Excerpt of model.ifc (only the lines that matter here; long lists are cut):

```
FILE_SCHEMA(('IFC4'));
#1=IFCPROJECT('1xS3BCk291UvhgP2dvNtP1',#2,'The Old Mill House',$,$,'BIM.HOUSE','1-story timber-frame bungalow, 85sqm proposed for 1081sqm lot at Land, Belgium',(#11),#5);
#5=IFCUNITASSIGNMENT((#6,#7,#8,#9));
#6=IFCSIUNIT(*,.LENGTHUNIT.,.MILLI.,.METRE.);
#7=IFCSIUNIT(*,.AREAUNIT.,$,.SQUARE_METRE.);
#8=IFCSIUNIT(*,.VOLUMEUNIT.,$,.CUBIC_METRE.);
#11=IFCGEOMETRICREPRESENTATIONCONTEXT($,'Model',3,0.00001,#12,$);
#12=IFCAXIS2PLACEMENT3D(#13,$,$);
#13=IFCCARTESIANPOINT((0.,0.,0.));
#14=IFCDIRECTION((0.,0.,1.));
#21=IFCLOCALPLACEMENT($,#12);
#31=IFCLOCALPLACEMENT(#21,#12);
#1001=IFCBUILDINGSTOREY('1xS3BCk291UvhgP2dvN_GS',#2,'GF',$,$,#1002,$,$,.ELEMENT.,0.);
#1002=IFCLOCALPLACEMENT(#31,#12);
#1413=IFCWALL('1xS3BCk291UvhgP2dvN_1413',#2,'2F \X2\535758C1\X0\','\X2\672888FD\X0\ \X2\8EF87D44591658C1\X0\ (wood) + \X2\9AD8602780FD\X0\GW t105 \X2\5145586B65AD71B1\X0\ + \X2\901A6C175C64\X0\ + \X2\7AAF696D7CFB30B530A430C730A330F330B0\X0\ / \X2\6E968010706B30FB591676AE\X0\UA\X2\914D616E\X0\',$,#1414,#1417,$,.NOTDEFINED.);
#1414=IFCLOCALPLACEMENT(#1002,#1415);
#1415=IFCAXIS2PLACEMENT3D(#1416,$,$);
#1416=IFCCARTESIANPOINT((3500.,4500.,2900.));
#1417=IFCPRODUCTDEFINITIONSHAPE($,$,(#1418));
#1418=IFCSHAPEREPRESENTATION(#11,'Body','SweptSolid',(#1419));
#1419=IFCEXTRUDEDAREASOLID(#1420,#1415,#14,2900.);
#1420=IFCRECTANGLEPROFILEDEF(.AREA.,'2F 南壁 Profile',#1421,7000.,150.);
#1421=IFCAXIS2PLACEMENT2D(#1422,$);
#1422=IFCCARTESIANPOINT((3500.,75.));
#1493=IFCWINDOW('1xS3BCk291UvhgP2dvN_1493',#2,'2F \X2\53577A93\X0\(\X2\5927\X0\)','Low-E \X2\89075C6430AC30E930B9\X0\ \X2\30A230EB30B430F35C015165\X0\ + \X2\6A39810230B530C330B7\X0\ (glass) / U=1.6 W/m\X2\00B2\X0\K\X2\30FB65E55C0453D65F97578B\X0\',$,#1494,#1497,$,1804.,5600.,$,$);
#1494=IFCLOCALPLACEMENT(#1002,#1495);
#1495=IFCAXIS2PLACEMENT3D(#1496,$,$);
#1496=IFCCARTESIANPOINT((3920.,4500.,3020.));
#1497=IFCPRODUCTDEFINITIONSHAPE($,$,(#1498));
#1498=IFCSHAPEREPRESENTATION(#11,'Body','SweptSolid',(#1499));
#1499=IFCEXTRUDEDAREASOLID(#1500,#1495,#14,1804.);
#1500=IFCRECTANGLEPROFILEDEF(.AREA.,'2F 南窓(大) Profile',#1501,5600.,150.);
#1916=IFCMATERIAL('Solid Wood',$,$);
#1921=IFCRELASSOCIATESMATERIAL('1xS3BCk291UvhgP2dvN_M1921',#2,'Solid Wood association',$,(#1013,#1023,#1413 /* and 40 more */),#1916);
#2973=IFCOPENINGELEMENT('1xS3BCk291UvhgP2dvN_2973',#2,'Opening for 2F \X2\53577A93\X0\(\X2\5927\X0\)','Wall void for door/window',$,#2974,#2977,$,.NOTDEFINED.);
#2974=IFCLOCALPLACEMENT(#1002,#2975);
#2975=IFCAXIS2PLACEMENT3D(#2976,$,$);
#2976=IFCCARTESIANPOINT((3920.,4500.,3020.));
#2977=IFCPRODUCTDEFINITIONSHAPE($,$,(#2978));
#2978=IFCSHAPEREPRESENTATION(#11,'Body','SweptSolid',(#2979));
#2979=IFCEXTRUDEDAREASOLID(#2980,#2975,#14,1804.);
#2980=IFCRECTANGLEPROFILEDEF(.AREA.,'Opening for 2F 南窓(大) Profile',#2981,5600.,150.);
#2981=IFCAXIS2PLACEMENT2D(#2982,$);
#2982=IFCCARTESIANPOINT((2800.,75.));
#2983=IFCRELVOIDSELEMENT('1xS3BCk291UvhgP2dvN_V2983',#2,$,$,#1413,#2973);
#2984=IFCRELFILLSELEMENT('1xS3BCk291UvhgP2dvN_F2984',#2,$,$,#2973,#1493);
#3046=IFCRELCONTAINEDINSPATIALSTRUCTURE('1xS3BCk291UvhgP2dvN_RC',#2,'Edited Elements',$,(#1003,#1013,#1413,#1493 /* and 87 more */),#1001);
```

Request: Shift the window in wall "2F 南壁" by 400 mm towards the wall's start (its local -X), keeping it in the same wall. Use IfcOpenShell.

```python
import ifcopenshell
import ifcopenshell.api.geometry
import ifcopenshell.util.placement
import ifcopenshell.util.unit

model = ifcopenshell.open("model.ifc")
unit_scale = ifcopenshell.util.unit.calculate_unit_scale(model)

window = model.by_guid("1xS3BCk291UvhgP2dvN_1493")
opening = window.FillsVoids[0].RelatingOpeningElement
wall = opening.VoidsElements[0].RelatingBuildingElement

wall_matrix = ifcopenshell.util.placement.get_local_placement(wall.ObjectPlacement)
shift = wall_matrix[:3, 0] * -0.4 / unit_scale
before = ifcopenshell.util.placement.get_local_placement(window.ObjectPlacement)[:3, 3].copy()

# The window is not placed relative to its opening, so move both.
for product in (opening, window):
    matrix = ifcopenshell.util.placement.get_local_placement(product.ObjectPlacement)
    matrix[:3, 3] += shift
    ifcopenshell.api.geometry.edit_object_placement(model, product=product, matrix=matrix, is_si=False)

after = ifcopenshell.util.placement.get_local_placement(window.ObjectPlacement)[:3, 3]
print("window moved by", (after - before).round(3) + 0.0)

model.write("model_edited.ifc")
```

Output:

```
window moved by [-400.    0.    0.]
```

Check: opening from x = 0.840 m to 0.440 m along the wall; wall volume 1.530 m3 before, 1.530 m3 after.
